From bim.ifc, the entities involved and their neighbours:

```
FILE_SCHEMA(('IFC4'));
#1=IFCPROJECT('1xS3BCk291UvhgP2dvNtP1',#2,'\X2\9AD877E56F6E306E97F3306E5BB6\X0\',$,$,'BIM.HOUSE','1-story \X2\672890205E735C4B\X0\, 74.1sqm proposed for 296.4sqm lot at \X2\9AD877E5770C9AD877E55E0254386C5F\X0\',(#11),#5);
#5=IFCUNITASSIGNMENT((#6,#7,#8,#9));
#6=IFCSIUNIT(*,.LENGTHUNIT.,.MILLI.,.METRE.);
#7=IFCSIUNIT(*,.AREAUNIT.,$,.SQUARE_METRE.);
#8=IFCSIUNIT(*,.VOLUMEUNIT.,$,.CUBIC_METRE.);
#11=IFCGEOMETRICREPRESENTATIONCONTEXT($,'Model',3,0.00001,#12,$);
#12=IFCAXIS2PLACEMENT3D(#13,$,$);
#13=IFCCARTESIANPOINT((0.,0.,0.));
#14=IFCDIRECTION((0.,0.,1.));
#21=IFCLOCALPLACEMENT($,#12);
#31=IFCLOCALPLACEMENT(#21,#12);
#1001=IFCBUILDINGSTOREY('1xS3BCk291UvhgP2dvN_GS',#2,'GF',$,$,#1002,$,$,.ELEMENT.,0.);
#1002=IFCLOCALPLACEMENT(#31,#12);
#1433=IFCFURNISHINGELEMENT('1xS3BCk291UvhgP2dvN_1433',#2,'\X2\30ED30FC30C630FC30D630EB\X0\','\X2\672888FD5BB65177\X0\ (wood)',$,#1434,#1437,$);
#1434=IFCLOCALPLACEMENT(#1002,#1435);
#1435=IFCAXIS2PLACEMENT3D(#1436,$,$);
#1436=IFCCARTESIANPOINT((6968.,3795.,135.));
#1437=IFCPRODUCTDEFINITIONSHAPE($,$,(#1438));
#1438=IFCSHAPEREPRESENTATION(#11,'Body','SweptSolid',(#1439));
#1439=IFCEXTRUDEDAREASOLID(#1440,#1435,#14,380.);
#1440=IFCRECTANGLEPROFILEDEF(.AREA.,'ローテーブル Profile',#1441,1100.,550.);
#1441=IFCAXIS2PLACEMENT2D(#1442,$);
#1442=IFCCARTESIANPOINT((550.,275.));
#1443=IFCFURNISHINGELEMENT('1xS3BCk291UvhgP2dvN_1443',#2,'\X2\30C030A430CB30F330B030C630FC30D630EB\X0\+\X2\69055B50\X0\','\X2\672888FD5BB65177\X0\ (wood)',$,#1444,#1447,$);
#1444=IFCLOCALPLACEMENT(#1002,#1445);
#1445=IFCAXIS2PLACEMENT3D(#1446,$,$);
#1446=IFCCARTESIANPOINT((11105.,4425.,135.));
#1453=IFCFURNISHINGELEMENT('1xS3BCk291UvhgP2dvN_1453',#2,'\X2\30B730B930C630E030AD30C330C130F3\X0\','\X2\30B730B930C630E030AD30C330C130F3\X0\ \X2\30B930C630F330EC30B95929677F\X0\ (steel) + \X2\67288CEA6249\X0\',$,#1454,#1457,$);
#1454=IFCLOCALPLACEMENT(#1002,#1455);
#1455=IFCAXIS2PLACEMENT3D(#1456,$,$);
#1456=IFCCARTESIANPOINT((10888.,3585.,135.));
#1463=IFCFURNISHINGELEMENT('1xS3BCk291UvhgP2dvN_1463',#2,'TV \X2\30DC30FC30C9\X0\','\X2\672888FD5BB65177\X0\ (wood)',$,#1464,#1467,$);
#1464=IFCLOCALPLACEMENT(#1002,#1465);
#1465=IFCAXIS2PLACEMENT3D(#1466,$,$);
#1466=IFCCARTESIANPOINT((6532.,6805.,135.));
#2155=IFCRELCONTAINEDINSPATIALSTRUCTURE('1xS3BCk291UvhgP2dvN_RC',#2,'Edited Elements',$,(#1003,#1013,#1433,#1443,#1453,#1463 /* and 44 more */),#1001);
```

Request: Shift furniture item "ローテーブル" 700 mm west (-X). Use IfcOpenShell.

```python
import ifcopenshell
import ifcopenshell.api.geometry
import ifcopenshell.util.placement
import ifcopenshell.util.unit

model = ifcopenshell.open("bim.ifc")
unit_scale = ifcopenshell.util.unit.calculate_unit_scale(model)

item = model.by_guid("1xS3BCk291UvhgP2dvN_1433")
matrix = ifcopenshell.util.placement.get_local_placement(item.ObjectPlacement)
matrix[0, 3] -= 0.7 / unit_scale
ifcopenshell.api.geometry.edit_object_placement(model, product=item, matrix=matrix, is_si=False)

print(ifcopenshell.util.placement.get_local_placement(item.ObjectPlacement).round(3) + 0.0)

model.write("bim_rev.ifc")
```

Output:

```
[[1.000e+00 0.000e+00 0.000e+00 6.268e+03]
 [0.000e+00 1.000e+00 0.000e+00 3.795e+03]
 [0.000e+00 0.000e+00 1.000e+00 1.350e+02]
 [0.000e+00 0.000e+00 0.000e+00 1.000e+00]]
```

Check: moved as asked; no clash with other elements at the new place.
